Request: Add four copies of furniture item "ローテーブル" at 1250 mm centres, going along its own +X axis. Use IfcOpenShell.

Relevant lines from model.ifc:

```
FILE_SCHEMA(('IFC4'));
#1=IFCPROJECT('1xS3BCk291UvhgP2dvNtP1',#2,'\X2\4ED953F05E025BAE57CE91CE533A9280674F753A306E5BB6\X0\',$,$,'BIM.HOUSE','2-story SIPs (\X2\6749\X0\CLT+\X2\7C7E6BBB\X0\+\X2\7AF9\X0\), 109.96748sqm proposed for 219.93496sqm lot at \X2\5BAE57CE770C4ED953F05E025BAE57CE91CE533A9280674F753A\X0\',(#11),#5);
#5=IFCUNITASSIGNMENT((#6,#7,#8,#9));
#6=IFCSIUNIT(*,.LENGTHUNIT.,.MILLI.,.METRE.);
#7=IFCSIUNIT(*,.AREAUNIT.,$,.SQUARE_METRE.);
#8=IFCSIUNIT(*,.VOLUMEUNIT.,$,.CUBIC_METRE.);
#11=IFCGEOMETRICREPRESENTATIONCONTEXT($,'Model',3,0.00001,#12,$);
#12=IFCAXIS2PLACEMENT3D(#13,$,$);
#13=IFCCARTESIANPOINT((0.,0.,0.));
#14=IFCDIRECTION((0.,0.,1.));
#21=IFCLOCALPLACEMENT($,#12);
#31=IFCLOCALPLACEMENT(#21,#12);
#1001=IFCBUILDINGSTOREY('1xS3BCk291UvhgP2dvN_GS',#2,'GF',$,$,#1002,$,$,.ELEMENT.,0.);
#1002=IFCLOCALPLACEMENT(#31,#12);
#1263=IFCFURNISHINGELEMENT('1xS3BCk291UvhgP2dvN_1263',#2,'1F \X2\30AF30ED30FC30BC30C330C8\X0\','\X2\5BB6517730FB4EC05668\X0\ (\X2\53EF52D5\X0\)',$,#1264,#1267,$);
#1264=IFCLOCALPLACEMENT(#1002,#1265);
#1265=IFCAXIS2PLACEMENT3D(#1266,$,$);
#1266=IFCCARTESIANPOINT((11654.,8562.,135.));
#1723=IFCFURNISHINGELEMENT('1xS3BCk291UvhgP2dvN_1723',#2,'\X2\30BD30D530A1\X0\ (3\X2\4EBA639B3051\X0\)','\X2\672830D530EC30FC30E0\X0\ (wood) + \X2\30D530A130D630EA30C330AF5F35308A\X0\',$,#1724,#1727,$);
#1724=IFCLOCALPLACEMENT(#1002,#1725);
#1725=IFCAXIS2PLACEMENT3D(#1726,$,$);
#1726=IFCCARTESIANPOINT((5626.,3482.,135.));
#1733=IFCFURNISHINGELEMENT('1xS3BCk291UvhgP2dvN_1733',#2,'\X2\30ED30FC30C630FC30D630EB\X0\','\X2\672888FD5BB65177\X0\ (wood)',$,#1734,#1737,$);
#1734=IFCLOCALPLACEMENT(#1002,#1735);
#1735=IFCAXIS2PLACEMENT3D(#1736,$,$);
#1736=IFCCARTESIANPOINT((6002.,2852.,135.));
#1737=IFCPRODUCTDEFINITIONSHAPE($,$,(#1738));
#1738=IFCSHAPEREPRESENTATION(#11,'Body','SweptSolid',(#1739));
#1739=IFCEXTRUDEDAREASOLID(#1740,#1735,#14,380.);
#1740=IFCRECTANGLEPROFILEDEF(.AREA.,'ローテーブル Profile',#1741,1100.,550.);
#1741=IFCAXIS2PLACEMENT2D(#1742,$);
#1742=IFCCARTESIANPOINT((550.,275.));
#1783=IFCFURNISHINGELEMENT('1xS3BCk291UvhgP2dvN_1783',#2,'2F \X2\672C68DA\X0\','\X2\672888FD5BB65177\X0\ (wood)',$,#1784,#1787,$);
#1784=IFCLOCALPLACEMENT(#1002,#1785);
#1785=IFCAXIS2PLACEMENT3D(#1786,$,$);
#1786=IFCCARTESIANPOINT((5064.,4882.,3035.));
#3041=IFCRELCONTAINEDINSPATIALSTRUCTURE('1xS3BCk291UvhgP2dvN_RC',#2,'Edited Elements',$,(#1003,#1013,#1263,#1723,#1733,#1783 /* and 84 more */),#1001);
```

```python
import ifcopenshell
import ifcopenshell.api.geometry
import ifcopenshell.api.root
import ifcopenshell.util.element
import ifcopenshell.util.placement
import ifcopenshell.util.unit

model = ifcopenshell.open("model.ifc")
unit_scale = ifcopenshell.util.unit.calculate_unit_scale(model)


def reuse_history(source, copy):
    """copy_class also copies each property set's owner history, people and application; keep the originals."""
    for rel in copy.IsDefinedBy:
        if rel.is_a("IfcRelDefinesByProperties") and (history := rel.RelatingPropertyDefinition.OwnerHistory):
            rel.RelatingPropertyDefinition.OwnerHistory = source.OwnerHistory
            ifcopenshell.util.element.remove_deep2(model, history)


source = model.by_guid("1xS3BCk291UvhgP2dvN_1733")
base = ifcopenshell.util.placement.get_local_placement(source.ObjectPlacement)
step = base[:3, 0] * 1.25 / unit_scale

for i in range(1, 5):
    copy = ifcopenshell.api.root.copy_class(model, product=source)
    copy.Representation = ifcopenshell.util.element.copy_deep(
        model, source.Representation, exclude=["IfcGeometricRepresentationContext", "IfcRepresentationMap"]
    )
    reuse_history(source, copy)
    matrix = base.copy()
    matrix[:3, 3] += i * step
    print("added at", matrix[:3, 3].round(3) + 0.0)
    ifcopenshell.api.geometry.edit_object_placement(model, product=copy, matrix=matrix, is_si=False)

model.write("model-out.ifc")
```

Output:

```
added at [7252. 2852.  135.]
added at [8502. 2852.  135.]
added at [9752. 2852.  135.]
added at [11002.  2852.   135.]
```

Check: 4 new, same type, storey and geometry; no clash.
